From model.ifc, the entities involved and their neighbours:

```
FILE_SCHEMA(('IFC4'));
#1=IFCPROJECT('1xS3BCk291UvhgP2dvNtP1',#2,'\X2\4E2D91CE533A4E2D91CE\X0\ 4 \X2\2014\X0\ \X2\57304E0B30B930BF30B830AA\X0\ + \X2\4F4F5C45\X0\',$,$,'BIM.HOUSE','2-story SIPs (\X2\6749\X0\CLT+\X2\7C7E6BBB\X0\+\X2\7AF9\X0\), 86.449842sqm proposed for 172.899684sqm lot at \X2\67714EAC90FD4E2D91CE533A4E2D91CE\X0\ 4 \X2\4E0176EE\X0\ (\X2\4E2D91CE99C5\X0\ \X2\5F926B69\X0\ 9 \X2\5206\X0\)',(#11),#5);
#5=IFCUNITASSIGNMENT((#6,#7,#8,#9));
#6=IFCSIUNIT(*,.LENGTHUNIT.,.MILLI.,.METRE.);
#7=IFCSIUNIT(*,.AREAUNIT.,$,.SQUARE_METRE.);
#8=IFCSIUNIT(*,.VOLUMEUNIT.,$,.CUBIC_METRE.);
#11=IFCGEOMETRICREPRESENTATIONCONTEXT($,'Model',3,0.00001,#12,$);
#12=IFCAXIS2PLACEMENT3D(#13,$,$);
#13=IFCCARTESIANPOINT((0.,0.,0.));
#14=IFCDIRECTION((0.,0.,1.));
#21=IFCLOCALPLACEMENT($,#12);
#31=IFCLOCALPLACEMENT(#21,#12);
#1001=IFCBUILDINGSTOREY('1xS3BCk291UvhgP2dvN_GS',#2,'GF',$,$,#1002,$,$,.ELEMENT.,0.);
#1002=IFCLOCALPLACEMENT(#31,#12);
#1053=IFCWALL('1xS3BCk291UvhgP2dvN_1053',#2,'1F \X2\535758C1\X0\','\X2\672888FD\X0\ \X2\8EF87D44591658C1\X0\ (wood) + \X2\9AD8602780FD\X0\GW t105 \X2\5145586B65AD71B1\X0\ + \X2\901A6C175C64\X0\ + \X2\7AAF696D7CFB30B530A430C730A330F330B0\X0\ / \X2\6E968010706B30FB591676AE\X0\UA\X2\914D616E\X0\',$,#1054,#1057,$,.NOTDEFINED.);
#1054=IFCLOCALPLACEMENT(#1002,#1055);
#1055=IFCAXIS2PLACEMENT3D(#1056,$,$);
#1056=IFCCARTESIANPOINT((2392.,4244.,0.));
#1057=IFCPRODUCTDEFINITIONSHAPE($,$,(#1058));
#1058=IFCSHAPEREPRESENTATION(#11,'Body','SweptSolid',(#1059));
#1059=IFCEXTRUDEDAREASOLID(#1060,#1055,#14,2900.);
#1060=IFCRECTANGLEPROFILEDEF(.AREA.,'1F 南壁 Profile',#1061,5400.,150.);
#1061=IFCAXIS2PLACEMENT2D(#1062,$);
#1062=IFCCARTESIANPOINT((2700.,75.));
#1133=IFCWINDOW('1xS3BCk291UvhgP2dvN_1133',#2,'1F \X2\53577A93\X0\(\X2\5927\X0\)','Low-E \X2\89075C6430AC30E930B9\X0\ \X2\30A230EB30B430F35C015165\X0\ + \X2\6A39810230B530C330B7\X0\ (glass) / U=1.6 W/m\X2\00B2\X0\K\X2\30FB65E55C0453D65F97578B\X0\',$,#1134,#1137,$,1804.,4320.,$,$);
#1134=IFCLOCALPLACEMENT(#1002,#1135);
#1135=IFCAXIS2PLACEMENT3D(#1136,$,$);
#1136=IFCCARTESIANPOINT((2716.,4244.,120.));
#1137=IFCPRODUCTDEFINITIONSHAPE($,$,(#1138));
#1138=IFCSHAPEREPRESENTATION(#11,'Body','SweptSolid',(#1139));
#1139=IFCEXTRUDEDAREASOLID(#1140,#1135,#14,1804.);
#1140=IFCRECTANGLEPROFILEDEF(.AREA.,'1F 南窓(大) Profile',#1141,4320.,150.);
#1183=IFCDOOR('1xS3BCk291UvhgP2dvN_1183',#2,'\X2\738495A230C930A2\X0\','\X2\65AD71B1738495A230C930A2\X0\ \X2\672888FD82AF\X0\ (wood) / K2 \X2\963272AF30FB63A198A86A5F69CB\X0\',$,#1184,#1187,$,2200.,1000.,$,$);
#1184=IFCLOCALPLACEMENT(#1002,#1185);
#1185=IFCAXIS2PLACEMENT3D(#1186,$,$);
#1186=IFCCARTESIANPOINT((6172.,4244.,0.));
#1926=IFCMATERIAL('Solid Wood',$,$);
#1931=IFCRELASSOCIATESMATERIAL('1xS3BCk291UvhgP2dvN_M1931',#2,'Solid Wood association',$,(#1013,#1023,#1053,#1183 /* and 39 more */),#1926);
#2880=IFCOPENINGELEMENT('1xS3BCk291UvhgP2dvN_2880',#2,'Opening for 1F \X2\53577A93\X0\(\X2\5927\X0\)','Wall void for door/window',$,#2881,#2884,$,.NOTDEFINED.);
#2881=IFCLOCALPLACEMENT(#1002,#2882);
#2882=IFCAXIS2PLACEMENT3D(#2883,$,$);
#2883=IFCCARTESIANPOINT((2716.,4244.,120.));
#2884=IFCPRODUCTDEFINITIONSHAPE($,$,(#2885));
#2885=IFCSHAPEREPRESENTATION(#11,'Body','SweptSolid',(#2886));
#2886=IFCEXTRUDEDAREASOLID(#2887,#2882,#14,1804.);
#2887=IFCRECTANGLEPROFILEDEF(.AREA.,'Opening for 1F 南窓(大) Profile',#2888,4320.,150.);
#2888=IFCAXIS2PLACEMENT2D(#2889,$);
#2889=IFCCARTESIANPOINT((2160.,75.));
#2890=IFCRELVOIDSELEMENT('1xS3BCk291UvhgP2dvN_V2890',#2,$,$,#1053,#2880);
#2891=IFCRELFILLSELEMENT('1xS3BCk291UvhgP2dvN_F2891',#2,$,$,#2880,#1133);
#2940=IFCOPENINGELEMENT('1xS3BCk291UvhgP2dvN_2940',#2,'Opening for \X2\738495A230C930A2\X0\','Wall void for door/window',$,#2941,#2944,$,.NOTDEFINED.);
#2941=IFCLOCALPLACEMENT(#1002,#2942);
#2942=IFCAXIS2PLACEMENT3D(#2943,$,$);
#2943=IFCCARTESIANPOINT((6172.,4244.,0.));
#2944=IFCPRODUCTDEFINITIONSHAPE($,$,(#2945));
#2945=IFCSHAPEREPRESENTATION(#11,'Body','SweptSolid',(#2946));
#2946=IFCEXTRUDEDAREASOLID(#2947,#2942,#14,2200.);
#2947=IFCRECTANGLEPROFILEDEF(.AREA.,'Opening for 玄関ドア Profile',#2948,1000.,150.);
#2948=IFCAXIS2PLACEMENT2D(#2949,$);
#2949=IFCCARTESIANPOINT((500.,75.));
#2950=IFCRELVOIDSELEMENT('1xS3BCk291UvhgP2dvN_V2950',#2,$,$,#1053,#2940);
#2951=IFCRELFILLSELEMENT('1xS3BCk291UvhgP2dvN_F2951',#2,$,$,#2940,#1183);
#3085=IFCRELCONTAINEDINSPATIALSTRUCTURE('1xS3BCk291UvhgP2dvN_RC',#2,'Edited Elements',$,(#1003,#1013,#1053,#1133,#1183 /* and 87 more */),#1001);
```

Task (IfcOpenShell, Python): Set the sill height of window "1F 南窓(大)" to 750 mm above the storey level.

```python
import numpy as np
import ifcopenshell
import ifcopenshell.api.geometry
import ifcopenshell.geom
import ifcopenshell.util.element
import ifcopenshell.util.placement
import ifcopenshell.util.shape
import ifcopenshell.util.unit

model = ifcopenshell.open("model.ifc")
unit_scale = ifcopenshell.util.unit.calculate_unit_scale(model)

window = model.by_guid("1xS3BCk291UvhgP2dvN_1133")
opening = window.FillsVoids[0].RelatingOpeningElement
storey = ifcopenshell.util.element.get_container(window, ifc_class="IfcBuildingStorey")
level = ifcopenshell.util.placement.get_local_placement(storey.ObjectPlacement)[2, 3]

# The opening's origin need not be at the sill, so measure its lowest point.
shape = ifcopenshell.geom.create_shape(ifcopenshell.geom.settings(), opening)
bottom = ifcopenshell.util.shape.get_shape_bottom_elevation(shape, shape.geometry) / unit_scale
dz = level + 750.0 - bottom

shift = np.array([0.0, 0.0, dz])
# The window is not placed relative to its opening, so move both.
for product in (opening, window):
    matrix = ifcopenshell.util.placement.get_local_placement(product.ObjectPlacement)
    matrix[:3, 3] += shift
    ifcopenshell.api.geometry.edit_object_placement(model, product=product, matrix=matrix, is_si=False)

print(f"moved by {dz * unit_scale:+.3f} m")

model.write("model_updated.ifc")
```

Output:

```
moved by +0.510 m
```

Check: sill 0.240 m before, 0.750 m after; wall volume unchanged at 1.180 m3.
